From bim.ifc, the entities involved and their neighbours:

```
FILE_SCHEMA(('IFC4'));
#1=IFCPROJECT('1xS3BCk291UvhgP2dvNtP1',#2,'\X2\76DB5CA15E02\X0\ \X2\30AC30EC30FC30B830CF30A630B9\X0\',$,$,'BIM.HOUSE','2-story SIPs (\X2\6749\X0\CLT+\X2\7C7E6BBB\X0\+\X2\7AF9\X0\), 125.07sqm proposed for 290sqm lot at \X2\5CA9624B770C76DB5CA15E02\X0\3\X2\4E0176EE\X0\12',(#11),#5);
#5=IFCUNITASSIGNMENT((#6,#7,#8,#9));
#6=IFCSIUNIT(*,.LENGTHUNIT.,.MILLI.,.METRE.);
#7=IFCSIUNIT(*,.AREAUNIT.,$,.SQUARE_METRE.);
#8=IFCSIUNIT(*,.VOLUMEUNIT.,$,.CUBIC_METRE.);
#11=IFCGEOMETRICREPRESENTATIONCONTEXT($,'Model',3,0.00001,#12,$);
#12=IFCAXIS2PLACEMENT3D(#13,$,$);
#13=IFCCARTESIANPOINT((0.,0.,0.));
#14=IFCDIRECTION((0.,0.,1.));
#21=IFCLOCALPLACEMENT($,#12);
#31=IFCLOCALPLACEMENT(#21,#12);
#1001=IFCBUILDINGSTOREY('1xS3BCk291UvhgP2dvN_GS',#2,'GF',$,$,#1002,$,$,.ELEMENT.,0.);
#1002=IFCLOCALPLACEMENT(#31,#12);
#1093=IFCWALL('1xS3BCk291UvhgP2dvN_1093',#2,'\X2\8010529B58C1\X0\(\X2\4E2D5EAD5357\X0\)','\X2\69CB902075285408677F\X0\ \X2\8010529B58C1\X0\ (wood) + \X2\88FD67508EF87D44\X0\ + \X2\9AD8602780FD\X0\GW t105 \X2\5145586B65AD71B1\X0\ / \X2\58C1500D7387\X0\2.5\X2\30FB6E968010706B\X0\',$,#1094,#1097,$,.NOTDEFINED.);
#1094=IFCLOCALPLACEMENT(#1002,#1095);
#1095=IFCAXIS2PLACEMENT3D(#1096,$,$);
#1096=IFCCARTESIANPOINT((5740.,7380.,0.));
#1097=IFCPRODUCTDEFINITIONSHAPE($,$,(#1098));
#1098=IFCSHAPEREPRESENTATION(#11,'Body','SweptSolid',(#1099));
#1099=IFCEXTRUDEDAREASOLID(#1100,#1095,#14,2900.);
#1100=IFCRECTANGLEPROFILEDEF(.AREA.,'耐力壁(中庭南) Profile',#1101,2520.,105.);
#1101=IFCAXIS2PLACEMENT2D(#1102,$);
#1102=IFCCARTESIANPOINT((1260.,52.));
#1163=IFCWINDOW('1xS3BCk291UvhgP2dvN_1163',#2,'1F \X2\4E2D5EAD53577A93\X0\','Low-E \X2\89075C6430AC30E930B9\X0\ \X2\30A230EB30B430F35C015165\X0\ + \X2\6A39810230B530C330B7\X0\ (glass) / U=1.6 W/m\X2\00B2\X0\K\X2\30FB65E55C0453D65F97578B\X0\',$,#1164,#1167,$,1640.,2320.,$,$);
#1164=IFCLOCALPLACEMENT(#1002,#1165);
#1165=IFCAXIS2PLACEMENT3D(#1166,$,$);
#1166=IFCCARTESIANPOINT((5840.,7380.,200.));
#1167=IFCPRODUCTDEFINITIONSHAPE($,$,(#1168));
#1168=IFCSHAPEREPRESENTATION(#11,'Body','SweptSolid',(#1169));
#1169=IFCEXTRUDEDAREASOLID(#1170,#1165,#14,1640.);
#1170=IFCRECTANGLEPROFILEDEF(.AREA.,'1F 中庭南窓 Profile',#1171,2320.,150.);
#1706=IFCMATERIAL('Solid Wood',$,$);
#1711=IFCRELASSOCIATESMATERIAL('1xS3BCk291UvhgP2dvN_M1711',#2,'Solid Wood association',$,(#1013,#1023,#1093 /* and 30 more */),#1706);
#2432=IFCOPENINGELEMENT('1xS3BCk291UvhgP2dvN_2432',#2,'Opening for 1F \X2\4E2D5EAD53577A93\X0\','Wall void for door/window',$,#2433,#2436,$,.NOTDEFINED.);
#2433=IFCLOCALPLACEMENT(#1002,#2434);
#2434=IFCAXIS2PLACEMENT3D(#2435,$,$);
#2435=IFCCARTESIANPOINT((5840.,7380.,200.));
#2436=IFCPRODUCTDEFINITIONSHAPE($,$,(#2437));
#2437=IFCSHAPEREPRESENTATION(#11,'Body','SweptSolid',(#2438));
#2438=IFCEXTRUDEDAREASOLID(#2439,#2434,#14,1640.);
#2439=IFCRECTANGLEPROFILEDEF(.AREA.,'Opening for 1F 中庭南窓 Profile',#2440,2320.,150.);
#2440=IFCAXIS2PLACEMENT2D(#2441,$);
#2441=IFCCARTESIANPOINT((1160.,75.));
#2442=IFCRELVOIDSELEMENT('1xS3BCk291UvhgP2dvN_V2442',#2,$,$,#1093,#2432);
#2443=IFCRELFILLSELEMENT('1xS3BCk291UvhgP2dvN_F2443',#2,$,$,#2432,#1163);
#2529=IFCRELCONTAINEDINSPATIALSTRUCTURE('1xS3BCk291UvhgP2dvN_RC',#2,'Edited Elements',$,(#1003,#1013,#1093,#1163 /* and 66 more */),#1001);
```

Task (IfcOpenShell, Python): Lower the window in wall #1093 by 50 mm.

```python
import numpy as np
import ifcopenshell
import ifcopenshell.api.geometry
import ifcopenshell.util.placement
import ifcopenshell.util.unit

model = ifcopenshell.open("bim.ifc")
unit_scale = ifcopenshell.util.unit.calculate_unit_scale(model)

window = model.by_id(1163)
opening = window.FillsVoids[0].RelatingOpeningElement
dz = -0.05 / unit_scale

shift = np.array([0.0, 0.0, dz])
# The window is not placed relative to its opening, so move both.
for product in (opening, window):
    matrix = ifcopenshell.util.placement.get_local_placement(product.ObjectPlacement)
    matrix[:3, 3] += shift
    ifcopenshell.api.geometry.edit_object_placement(model, product=product, matrix=matrix, is_si=False)

print(f"moved by {dz * unit_scale:+.3f} m")

model.write("bim_rev.ifc")
```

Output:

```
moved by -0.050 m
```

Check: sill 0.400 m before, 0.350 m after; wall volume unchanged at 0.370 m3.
